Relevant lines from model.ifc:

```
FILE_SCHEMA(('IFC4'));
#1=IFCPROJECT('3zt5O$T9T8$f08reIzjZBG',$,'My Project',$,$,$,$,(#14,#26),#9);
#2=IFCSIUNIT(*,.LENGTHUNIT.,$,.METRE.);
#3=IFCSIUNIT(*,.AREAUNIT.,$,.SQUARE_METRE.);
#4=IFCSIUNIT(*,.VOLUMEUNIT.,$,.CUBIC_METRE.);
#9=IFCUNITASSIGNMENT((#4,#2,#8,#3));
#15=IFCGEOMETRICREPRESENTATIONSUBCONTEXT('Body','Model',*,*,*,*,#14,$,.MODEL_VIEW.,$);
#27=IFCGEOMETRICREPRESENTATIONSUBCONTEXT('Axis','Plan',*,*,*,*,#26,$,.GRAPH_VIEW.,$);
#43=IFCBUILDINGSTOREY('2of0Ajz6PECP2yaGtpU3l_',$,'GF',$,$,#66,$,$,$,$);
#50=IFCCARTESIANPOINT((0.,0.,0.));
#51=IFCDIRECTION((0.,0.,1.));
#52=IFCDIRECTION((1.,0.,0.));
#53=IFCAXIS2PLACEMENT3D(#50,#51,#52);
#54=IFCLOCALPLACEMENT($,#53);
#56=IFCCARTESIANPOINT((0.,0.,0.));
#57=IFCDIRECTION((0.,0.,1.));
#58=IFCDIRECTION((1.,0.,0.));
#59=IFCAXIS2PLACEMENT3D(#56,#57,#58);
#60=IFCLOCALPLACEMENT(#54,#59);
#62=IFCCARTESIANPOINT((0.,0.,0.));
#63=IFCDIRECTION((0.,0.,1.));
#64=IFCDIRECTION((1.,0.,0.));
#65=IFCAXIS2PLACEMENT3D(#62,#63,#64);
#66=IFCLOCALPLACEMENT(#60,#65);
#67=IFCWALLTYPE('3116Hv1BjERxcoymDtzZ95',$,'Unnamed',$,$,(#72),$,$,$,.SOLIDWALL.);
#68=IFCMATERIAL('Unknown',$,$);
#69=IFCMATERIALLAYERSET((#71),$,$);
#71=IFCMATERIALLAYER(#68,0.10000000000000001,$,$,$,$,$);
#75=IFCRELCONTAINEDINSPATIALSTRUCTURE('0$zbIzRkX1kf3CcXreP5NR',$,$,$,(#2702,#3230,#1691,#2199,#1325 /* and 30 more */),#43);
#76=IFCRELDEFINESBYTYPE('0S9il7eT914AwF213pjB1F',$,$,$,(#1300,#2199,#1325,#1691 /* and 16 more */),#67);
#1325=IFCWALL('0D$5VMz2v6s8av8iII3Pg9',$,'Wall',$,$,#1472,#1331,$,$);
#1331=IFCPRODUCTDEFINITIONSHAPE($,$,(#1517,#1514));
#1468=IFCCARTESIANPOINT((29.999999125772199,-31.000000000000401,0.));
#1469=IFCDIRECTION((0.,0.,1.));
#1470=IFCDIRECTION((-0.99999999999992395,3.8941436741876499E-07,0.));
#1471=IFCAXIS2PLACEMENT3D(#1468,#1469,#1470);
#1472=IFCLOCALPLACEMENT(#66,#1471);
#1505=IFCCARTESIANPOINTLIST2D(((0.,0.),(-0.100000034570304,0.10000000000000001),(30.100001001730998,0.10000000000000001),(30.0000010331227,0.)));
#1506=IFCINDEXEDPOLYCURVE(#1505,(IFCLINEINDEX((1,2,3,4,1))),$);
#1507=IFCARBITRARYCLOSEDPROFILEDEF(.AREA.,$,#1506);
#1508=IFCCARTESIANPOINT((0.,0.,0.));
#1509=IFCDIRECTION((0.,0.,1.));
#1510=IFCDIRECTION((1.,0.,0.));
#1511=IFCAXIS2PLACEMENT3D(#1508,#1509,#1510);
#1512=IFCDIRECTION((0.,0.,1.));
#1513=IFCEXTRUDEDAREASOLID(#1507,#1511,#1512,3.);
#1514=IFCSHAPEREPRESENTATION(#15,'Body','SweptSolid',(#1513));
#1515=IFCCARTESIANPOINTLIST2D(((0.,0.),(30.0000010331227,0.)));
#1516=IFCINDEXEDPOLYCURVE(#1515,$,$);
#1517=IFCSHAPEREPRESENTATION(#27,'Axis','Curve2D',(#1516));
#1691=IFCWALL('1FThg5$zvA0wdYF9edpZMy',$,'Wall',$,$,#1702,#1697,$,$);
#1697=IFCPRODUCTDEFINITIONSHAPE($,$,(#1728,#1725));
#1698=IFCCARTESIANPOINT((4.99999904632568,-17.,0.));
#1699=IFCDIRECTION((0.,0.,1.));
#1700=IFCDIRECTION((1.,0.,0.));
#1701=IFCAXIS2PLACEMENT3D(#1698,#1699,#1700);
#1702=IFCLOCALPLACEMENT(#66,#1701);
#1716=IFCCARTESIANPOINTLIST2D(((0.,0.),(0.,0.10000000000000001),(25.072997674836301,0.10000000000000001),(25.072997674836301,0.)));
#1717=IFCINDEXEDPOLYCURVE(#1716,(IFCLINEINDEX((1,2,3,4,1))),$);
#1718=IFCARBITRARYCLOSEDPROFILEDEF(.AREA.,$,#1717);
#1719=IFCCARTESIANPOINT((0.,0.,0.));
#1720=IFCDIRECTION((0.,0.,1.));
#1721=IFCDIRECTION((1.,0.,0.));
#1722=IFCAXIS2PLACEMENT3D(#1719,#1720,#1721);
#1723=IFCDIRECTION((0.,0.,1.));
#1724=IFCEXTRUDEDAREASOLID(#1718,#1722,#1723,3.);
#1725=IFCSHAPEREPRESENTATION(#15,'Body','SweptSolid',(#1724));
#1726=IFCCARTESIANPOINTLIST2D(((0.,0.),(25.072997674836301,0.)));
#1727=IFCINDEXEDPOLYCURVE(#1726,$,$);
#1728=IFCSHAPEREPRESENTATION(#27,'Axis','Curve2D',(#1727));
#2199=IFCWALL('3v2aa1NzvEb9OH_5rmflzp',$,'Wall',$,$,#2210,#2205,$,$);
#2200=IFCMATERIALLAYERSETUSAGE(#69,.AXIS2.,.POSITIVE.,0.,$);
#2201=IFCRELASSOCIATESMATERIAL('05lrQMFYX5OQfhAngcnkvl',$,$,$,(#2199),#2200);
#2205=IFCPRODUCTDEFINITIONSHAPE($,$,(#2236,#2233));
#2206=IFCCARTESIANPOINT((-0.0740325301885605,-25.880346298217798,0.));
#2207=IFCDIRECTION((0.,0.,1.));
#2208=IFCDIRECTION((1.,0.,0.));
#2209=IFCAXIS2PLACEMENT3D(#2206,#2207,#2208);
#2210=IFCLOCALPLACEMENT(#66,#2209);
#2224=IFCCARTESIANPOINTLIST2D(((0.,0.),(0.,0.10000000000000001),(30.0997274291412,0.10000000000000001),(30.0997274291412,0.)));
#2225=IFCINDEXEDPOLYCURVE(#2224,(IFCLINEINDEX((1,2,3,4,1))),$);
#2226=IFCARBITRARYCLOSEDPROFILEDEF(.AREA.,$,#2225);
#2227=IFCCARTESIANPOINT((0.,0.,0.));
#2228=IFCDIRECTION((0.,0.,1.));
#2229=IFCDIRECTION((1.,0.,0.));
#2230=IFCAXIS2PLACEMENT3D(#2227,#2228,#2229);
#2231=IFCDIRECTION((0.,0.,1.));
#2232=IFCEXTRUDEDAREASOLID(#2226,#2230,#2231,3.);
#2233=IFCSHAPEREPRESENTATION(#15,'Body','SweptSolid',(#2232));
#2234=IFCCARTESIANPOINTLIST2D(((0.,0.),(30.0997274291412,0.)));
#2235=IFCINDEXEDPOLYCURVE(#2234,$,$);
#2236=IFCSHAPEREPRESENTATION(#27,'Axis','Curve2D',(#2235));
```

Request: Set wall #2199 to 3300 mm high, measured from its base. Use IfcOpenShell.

```python
import ifcopenshell
import ifcopenshell.geom
import ifcopenshell.util.representation
import ifcopenshell.util.shape
import ifcopenshell.util.unit

model = ifcopenshell.open("model.ifc")
unit_scale = ifcopenshell.util.unit.calculate_unit_scale(model)
settings = ifcopenshell.geom.settings()


def volume(element):
    """Net volume in cubic metres, openings subtracted."""
    shape = ifcopenshell.geom.create_shape(settings, element)
    return ifcopenshell.util.shape.get_volume(shape.geometry)


wall = model.by_id(2199)
before = volume(wall)

body = ifcopenshell.util.representation.get_representation(wall, "Model", "Body")
solid = body.Items[0]
old_height = solid.Depth
solid.Depth = 3.3 / unit_scale
after = volume(wall)

print(f"height {old_height:g} -> {solid.Depth:g}, volume {before:.3f} -> {after:.3f} m3")

model.write("model_v2.ifc")
```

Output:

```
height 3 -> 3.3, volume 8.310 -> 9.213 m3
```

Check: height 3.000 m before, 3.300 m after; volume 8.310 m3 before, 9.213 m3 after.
